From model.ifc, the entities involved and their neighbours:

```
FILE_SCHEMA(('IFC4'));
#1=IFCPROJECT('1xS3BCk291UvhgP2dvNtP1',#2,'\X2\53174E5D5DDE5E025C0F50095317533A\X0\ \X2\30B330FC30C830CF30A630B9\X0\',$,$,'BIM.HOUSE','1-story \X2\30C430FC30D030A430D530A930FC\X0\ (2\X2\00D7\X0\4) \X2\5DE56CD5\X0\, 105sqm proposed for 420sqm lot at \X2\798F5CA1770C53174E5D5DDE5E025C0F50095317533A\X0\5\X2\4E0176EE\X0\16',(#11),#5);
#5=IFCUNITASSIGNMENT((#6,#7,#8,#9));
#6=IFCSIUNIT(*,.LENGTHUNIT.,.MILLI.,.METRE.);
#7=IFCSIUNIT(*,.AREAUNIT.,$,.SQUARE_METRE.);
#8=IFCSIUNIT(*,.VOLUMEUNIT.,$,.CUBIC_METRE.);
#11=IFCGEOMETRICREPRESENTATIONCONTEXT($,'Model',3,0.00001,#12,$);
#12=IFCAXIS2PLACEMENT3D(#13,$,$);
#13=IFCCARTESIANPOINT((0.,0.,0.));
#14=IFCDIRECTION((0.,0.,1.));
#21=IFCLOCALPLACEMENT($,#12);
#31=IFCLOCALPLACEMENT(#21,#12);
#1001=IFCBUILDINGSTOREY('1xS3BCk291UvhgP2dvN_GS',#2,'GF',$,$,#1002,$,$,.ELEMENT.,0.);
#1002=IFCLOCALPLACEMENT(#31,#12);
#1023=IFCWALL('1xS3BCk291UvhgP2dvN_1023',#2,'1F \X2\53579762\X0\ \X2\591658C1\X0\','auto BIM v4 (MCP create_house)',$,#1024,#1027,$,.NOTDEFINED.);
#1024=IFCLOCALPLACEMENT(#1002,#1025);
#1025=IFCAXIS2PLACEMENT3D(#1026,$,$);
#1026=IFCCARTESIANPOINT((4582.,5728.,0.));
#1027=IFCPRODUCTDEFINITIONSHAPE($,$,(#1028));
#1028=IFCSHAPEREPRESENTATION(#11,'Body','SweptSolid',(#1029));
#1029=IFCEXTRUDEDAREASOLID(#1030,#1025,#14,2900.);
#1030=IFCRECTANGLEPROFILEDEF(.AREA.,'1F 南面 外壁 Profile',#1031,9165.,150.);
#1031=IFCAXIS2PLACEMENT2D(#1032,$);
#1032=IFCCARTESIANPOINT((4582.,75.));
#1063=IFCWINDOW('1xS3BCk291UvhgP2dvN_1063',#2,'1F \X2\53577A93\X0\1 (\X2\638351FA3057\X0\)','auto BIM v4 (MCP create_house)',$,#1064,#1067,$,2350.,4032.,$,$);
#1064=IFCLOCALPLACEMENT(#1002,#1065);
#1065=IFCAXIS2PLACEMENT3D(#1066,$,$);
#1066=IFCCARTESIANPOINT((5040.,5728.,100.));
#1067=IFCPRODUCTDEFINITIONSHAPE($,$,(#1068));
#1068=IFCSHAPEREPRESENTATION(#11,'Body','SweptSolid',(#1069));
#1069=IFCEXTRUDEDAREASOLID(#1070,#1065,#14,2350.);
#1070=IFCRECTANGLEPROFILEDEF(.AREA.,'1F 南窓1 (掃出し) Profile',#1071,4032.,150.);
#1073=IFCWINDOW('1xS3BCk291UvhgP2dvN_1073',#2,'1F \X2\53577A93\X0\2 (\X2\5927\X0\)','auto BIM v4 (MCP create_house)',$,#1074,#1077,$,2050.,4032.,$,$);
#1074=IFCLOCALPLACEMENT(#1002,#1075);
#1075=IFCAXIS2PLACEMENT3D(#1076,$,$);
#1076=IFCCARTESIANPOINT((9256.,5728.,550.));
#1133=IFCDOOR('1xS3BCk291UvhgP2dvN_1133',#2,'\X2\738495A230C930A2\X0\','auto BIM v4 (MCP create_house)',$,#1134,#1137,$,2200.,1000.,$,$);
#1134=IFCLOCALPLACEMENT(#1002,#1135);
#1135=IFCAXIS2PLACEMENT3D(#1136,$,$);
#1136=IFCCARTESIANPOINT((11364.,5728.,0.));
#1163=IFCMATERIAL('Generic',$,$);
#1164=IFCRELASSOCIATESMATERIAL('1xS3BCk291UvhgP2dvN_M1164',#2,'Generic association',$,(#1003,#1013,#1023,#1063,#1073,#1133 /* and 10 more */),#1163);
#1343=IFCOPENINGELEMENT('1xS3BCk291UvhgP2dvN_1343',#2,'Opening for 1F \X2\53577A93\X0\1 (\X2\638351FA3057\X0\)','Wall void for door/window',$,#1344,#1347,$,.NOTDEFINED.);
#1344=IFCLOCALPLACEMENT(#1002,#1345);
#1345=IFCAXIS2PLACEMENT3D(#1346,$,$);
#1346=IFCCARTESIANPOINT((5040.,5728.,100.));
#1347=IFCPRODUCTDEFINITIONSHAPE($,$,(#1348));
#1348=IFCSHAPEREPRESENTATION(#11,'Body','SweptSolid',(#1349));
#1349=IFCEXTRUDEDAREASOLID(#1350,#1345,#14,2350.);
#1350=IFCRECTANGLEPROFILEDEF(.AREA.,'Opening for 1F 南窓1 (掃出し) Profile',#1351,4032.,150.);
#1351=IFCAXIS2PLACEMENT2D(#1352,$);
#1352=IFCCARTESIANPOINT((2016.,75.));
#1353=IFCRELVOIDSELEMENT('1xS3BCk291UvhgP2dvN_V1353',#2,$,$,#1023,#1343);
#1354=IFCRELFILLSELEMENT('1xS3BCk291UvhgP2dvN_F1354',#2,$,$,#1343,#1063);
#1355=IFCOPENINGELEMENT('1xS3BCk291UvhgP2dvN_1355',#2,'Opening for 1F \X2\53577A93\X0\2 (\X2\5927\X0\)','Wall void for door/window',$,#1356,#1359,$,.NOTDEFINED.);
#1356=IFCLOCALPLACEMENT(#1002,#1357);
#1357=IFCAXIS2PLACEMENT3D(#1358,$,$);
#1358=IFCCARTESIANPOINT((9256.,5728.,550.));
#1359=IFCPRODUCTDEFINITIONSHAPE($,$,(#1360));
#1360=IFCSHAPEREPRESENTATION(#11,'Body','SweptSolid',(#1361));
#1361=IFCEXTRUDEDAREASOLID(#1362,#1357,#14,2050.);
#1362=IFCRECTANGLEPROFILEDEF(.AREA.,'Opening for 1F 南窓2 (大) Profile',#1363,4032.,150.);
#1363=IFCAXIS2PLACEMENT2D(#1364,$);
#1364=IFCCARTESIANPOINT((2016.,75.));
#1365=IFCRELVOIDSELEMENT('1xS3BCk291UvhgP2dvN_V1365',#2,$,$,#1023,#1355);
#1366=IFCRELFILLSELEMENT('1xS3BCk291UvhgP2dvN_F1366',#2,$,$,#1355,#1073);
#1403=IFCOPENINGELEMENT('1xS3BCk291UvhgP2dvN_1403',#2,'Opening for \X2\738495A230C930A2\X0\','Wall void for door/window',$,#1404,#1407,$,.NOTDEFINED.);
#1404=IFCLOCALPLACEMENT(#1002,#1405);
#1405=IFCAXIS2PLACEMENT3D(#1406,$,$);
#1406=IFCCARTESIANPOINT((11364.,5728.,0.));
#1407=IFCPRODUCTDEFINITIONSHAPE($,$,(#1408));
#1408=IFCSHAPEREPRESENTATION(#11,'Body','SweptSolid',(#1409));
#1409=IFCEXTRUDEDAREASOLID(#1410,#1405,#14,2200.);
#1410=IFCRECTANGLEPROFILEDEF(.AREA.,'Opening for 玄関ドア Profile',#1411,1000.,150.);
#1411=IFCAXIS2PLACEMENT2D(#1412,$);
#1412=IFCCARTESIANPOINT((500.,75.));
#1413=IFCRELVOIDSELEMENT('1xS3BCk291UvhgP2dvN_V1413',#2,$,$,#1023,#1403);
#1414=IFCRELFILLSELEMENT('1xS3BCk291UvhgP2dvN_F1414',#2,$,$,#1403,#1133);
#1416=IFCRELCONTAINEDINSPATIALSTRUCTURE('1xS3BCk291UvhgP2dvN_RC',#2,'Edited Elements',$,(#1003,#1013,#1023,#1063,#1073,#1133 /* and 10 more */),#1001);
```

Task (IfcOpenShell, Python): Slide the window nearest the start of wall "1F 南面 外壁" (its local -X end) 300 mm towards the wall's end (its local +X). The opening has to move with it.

```python
import ifcopenshell
import ifcopenshell.api.geometry
import ifcopenshell.util.placement

model = ifcopenshell.open("model.ifc")

window = model.by_guid("1xS3BCk291UvhgP2dvN_1063")
opening = window.FillsVoids[0].RelatingOpeningElement
wall = opening.VoidsElements[0].RelatingBuildingElement

wall_matrix = ifcopenshell.util.placement.get_local_placement(wall.ObjectPlacement)
shift = wall_matrix[:3, 0] * 300.0
before = ifcopenshell.util.placement.get_local_placement(window.ObjectPlacement)[:3, 3].copy()

# The window is not placed relative to its opening, so move both.
for product in (opening, window):
    matrix = ifcopenshell.util.placement.get_local_placement(product.ObjectPlacement)
    matrix[:3, 3] += shift
    ifcopenshell.api.geometry.edit_object_placement(model, product=product, matrix=matrix, is_si=False)

after = ifcopenshell.util.placement.get_local_placement(window.ObjectPlacement)[:3, 3]
print("window moved by", (after - before).round(3) + 0.0)

model.write("model_updated.ifc")
```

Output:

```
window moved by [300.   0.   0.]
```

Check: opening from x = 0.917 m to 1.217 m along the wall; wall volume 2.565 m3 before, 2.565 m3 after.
